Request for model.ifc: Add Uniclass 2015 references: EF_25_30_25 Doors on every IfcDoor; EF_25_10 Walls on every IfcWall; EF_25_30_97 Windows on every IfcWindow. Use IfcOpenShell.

First a look at what the model holds.

```python
import ifcopenshell

model = ifcopenshell.open("model.ifc")
print(model.schema)
print("classifications:", [c.Name for c in model.by_type("IfcClassification")])
for ifc_class in ("IfcDoor", "IfcRoof", "IfcStair", "IfcWall", "IfcWindow"):
    print(ifc_class, len(model.by_type(ifc_class)))
```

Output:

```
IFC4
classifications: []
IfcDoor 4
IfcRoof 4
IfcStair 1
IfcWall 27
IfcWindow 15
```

```python
import ifcopenshell
import ifcopenshell.api.classification

model = ifcopenshell.open("model.ifc")

system = ifcopenshell.api.classification.add_classification(model, classification="Uniclass 2015")

codes = {
    "IfcDoor": ("EF_25_30_25", "Doors"),
    "IfcWall": ("EF_25_10", "Walls"),
    "IfcWindow": ("EF_25_30_97", "Windows"),
}
for ifc_class, (code, name) in codes.items():
    products = model.by_type(ifc_class)
    ifcopenshell.api.classification.add_reference(
        model, products=products, classification=system, identification=code, name=name
    )
    print(code, len(products))

model.write("model_updated.ifc")
```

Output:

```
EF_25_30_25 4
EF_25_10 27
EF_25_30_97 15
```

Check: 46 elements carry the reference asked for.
